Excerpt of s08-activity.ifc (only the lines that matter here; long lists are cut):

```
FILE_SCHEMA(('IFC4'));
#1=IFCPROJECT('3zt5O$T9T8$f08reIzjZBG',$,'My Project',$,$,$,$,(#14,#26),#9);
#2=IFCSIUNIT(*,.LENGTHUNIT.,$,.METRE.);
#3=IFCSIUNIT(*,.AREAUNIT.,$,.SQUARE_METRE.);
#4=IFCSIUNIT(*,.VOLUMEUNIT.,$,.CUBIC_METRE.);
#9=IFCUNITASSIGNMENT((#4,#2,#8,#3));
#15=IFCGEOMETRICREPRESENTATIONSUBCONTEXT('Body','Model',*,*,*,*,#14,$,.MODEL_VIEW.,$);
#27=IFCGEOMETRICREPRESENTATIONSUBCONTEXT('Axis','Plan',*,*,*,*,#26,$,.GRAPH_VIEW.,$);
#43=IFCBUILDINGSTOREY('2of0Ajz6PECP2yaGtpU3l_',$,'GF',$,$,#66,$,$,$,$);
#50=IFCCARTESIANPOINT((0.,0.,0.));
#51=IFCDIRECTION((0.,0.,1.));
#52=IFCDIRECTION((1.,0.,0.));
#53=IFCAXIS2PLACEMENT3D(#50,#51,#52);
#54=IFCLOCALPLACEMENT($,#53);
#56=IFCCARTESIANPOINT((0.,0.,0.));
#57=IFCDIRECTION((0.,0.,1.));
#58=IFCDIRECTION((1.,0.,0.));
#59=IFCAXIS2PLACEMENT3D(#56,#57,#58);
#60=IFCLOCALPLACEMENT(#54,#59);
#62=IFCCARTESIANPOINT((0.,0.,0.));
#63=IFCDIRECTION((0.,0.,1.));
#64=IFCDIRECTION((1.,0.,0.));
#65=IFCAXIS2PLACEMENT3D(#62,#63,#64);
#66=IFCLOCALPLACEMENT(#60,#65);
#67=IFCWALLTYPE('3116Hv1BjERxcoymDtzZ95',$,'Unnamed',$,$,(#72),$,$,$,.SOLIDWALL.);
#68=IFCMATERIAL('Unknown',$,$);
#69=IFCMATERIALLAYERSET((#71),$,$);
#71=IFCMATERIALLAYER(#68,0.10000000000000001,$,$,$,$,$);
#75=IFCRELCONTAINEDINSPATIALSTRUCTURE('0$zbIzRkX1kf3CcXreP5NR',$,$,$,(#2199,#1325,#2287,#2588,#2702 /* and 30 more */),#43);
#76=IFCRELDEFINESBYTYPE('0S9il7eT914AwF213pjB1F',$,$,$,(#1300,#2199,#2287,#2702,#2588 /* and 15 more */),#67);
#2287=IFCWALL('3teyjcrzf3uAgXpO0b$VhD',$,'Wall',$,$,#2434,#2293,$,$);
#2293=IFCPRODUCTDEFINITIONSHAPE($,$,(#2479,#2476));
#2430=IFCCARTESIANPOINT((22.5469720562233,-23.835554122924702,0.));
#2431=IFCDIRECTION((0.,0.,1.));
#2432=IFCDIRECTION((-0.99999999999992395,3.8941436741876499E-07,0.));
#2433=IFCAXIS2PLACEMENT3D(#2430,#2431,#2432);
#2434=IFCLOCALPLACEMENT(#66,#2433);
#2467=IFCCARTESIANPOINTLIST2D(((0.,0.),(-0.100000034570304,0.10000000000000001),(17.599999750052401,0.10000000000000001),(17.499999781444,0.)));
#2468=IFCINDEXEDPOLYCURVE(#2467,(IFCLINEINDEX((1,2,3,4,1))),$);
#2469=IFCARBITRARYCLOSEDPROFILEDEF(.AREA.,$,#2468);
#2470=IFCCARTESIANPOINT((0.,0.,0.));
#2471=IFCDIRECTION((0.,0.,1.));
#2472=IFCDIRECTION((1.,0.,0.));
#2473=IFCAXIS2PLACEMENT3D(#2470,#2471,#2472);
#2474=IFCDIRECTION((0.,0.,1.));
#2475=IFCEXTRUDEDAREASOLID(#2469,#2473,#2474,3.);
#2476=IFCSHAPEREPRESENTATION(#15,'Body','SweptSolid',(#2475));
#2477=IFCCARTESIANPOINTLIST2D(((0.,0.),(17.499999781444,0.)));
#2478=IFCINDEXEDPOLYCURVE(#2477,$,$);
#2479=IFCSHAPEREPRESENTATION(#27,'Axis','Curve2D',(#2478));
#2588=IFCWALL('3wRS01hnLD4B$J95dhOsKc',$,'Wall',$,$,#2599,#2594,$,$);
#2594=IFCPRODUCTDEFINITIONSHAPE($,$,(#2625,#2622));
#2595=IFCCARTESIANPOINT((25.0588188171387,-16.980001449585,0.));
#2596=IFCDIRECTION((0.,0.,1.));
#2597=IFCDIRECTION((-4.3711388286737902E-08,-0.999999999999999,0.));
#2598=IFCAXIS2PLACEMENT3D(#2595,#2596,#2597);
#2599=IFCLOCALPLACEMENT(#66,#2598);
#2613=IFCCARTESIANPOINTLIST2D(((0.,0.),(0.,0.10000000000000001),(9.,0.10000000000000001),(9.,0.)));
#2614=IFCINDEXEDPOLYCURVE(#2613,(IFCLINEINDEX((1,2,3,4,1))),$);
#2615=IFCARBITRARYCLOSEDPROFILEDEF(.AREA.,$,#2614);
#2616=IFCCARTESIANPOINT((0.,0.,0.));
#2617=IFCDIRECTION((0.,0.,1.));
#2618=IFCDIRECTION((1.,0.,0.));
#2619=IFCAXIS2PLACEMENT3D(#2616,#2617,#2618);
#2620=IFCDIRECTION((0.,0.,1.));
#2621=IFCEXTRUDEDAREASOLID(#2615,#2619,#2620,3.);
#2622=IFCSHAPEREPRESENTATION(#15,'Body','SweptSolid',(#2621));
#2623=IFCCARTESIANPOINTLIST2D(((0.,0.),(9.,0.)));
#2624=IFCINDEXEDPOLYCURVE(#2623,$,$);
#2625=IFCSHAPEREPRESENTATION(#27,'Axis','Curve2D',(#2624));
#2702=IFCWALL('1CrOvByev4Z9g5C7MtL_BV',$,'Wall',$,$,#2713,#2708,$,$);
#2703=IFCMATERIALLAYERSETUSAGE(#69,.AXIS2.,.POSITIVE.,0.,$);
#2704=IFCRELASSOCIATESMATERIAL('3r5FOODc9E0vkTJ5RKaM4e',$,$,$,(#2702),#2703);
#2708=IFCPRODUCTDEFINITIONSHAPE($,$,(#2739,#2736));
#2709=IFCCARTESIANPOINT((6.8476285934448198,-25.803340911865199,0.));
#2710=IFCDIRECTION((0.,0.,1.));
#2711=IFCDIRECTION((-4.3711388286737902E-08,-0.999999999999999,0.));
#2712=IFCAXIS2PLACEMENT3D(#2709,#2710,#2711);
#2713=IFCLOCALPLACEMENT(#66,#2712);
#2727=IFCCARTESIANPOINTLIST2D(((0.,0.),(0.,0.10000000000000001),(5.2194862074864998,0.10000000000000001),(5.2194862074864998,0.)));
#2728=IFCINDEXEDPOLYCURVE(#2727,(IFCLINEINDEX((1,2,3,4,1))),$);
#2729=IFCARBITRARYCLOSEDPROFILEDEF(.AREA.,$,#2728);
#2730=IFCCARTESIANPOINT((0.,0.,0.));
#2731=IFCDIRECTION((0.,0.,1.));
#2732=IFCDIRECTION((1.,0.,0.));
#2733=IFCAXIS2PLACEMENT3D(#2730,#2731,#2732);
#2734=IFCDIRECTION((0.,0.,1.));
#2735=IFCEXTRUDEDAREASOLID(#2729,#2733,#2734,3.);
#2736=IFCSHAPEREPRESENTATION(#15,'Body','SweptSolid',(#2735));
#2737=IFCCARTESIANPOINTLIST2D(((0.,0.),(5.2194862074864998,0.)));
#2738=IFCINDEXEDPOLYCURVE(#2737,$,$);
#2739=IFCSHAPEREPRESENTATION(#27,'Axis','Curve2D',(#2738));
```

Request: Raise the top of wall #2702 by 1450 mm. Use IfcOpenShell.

```python
import ifcopenshell
import ifcopenshell.geom
import ifcopenshell.util.representation
import ifcopenshell.util.shape

model = ifcopenshell.open("s08-activity.ifc")
settings = ifcopenshell.geom.settings()


def volume(element):
    """Net volume in cubic metres, openings subtracted."""
    shape = ifcopenshell.geom.create_shape(settings, element)
    return ifcopenshell.util.shape.get_volume(shape.geometry)


wall = model.by_guid("1CrOvByev4Z9g5C7MtL_BV")
before = volume(wall)

body = ifcopenshell.util.representation.get_representation(wall, "Model", "Body")
solid = body.Items[0]
old_height = solid.Depth
solid.Depth += 1.45
after = volume(wall)

print(f"height {old_height:g} -> {solid.Depth:g}, volume {before:.3f} -> {after:.3f} m3")

model.write("s08-activity_v2.ifc")
```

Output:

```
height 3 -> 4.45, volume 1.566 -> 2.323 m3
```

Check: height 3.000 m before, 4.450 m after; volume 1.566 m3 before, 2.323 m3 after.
